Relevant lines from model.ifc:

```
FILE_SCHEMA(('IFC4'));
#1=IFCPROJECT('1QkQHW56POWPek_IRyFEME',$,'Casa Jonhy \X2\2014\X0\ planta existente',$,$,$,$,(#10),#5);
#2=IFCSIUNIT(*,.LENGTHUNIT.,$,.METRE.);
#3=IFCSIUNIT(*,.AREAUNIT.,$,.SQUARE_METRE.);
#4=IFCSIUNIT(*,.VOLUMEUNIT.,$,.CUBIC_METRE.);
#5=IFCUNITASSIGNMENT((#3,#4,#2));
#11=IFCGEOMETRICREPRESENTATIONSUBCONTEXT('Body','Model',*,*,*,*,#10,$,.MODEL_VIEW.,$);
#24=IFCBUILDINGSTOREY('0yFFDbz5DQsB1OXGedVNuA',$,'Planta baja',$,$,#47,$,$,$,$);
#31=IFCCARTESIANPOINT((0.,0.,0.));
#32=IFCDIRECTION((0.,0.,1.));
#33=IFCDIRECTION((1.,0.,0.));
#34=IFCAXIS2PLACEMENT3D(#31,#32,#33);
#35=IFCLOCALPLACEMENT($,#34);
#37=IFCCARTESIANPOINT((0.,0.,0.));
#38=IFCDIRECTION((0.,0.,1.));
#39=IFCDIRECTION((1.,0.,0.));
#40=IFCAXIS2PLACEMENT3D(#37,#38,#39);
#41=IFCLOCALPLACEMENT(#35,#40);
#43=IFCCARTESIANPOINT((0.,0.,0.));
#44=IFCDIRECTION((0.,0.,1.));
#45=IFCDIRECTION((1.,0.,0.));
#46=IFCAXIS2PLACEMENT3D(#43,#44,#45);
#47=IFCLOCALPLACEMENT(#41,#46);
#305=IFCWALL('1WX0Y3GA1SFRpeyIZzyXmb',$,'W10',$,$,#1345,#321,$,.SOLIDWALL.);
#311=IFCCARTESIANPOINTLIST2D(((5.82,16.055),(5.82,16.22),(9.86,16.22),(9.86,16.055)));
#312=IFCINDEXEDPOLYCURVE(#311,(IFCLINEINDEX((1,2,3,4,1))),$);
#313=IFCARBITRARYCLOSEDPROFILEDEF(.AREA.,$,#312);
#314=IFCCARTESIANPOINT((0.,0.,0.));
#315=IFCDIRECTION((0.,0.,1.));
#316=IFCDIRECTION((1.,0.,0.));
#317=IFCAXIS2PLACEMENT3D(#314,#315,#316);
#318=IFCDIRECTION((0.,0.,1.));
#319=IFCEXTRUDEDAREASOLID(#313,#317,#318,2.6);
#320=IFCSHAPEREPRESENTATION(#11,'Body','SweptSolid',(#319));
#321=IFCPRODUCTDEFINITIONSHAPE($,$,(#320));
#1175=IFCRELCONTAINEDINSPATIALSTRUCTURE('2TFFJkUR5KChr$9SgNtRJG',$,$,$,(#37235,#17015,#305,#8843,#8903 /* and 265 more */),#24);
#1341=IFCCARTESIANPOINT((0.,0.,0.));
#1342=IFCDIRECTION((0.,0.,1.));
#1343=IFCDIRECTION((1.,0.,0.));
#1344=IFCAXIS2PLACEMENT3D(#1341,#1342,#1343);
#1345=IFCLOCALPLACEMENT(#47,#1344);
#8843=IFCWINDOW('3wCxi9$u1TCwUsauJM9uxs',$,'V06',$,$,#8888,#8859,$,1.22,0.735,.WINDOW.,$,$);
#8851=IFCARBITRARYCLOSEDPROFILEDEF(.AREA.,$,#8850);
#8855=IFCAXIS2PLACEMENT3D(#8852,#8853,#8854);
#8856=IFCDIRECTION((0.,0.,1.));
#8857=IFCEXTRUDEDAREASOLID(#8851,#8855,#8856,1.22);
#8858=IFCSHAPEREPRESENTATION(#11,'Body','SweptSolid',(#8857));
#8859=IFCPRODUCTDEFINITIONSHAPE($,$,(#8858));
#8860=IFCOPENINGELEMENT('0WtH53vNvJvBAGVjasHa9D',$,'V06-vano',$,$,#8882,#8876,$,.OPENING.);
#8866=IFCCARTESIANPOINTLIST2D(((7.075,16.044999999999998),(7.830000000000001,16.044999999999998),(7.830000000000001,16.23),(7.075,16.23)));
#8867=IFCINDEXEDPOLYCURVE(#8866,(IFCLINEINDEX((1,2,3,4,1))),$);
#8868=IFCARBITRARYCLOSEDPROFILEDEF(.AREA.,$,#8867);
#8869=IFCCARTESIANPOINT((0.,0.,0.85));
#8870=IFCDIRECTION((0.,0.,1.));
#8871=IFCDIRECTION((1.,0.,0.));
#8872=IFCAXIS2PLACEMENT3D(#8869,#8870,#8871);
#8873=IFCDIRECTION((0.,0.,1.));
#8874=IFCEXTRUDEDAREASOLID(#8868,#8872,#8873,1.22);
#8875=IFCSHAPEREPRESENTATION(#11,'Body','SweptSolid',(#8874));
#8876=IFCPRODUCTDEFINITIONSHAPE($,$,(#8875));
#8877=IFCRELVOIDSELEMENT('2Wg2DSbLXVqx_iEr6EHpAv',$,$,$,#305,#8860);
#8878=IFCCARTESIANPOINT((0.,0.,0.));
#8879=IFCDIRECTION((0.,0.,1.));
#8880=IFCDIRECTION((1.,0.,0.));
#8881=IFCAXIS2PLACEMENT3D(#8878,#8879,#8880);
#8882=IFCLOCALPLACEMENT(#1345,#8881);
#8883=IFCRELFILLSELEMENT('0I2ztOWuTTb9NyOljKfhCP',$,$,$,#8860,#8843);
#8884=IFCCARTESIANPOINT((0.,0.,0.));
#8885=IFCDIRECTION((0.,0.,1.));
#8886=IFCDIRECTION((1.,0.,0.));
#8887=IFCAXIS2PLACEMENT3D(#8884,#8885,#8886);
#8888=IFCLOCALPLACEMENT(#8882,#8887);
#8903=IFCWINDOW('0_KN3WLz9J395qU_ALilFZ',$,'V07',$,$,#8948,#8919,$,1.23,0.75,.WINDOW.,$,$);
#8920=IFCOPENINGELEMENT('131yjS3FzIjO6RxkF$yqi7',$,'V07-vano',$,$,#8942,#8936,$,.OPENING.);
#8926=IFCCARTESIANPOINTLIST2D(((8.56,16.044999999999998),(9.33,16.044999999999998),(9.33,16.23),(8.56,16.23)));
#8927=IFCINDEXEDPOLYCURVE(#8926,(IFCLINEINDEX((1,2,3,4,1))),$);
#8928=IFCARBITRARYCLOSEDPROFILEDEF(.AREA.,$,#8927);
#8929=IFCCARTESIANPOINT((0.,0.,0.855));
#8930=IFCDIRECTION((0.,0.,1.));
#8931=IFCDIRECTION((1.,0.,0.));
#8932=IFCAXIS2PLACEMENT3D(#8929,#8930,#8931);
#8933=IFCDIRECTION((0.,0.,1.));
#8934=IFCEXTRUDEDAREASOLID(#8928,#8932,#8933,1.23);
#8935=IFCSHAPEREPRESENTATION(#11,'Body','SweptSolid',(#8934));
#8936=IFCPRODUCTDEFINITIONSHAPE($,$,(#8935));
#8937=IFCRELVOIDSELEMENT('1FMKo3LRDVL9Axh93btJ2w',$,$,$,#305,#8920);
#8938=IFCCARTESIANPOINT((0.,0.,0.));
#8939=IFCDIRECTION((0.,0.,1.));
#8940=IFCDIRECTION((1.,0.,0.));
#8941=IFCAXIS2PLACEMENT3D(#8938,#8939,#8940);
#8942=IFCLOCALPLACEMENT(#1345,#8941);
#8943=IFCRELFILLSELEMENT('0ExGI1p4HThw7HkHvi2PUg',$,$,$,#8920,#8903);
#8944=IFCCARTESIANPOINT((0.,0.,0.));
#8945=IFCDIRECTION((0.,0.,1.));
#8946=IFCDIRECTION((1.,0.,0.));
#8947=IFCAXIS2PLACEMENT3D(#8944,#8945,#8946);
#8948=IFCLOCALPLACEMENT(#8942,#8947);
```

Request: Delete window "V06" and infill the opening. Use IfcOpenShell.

```python
import ifcopenshell
import ifcopenshell.api.feature
import ifcopenshell.api.root
import ifcopenshell.geom
import ifcopenshell.util.shape

model = ifcopenshell.open("model.ifc")
settings = ifcopenshell.geom.settings()


def volume(element):
    """Net volume in cubic metres, openings subtracted."""
    shape = ifcopenshell.geom.create_shape(settings, element)
    return ifcopenshell.util.shape.get_volume(shape.geometry)


window = model.by_id(8843)
opening = window.FillsVoids[0].RelatingOpeningElement
wall = opening.VoidsElements[0].RelatingBuildingElement
before = volume(wall)

ifcopenshell.api.root.remove_product(model, product=window)
ifcopenshell.api.feature.remove_feature(model, feature=opening)

after = volume(wall)

print(f"wall volume {before:.3f} -> {after:.3f} m3")

model.write("model_updated.ifc")
```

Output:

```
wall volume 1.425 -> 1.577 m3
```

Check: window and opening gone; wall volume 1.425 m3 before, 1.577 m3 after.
